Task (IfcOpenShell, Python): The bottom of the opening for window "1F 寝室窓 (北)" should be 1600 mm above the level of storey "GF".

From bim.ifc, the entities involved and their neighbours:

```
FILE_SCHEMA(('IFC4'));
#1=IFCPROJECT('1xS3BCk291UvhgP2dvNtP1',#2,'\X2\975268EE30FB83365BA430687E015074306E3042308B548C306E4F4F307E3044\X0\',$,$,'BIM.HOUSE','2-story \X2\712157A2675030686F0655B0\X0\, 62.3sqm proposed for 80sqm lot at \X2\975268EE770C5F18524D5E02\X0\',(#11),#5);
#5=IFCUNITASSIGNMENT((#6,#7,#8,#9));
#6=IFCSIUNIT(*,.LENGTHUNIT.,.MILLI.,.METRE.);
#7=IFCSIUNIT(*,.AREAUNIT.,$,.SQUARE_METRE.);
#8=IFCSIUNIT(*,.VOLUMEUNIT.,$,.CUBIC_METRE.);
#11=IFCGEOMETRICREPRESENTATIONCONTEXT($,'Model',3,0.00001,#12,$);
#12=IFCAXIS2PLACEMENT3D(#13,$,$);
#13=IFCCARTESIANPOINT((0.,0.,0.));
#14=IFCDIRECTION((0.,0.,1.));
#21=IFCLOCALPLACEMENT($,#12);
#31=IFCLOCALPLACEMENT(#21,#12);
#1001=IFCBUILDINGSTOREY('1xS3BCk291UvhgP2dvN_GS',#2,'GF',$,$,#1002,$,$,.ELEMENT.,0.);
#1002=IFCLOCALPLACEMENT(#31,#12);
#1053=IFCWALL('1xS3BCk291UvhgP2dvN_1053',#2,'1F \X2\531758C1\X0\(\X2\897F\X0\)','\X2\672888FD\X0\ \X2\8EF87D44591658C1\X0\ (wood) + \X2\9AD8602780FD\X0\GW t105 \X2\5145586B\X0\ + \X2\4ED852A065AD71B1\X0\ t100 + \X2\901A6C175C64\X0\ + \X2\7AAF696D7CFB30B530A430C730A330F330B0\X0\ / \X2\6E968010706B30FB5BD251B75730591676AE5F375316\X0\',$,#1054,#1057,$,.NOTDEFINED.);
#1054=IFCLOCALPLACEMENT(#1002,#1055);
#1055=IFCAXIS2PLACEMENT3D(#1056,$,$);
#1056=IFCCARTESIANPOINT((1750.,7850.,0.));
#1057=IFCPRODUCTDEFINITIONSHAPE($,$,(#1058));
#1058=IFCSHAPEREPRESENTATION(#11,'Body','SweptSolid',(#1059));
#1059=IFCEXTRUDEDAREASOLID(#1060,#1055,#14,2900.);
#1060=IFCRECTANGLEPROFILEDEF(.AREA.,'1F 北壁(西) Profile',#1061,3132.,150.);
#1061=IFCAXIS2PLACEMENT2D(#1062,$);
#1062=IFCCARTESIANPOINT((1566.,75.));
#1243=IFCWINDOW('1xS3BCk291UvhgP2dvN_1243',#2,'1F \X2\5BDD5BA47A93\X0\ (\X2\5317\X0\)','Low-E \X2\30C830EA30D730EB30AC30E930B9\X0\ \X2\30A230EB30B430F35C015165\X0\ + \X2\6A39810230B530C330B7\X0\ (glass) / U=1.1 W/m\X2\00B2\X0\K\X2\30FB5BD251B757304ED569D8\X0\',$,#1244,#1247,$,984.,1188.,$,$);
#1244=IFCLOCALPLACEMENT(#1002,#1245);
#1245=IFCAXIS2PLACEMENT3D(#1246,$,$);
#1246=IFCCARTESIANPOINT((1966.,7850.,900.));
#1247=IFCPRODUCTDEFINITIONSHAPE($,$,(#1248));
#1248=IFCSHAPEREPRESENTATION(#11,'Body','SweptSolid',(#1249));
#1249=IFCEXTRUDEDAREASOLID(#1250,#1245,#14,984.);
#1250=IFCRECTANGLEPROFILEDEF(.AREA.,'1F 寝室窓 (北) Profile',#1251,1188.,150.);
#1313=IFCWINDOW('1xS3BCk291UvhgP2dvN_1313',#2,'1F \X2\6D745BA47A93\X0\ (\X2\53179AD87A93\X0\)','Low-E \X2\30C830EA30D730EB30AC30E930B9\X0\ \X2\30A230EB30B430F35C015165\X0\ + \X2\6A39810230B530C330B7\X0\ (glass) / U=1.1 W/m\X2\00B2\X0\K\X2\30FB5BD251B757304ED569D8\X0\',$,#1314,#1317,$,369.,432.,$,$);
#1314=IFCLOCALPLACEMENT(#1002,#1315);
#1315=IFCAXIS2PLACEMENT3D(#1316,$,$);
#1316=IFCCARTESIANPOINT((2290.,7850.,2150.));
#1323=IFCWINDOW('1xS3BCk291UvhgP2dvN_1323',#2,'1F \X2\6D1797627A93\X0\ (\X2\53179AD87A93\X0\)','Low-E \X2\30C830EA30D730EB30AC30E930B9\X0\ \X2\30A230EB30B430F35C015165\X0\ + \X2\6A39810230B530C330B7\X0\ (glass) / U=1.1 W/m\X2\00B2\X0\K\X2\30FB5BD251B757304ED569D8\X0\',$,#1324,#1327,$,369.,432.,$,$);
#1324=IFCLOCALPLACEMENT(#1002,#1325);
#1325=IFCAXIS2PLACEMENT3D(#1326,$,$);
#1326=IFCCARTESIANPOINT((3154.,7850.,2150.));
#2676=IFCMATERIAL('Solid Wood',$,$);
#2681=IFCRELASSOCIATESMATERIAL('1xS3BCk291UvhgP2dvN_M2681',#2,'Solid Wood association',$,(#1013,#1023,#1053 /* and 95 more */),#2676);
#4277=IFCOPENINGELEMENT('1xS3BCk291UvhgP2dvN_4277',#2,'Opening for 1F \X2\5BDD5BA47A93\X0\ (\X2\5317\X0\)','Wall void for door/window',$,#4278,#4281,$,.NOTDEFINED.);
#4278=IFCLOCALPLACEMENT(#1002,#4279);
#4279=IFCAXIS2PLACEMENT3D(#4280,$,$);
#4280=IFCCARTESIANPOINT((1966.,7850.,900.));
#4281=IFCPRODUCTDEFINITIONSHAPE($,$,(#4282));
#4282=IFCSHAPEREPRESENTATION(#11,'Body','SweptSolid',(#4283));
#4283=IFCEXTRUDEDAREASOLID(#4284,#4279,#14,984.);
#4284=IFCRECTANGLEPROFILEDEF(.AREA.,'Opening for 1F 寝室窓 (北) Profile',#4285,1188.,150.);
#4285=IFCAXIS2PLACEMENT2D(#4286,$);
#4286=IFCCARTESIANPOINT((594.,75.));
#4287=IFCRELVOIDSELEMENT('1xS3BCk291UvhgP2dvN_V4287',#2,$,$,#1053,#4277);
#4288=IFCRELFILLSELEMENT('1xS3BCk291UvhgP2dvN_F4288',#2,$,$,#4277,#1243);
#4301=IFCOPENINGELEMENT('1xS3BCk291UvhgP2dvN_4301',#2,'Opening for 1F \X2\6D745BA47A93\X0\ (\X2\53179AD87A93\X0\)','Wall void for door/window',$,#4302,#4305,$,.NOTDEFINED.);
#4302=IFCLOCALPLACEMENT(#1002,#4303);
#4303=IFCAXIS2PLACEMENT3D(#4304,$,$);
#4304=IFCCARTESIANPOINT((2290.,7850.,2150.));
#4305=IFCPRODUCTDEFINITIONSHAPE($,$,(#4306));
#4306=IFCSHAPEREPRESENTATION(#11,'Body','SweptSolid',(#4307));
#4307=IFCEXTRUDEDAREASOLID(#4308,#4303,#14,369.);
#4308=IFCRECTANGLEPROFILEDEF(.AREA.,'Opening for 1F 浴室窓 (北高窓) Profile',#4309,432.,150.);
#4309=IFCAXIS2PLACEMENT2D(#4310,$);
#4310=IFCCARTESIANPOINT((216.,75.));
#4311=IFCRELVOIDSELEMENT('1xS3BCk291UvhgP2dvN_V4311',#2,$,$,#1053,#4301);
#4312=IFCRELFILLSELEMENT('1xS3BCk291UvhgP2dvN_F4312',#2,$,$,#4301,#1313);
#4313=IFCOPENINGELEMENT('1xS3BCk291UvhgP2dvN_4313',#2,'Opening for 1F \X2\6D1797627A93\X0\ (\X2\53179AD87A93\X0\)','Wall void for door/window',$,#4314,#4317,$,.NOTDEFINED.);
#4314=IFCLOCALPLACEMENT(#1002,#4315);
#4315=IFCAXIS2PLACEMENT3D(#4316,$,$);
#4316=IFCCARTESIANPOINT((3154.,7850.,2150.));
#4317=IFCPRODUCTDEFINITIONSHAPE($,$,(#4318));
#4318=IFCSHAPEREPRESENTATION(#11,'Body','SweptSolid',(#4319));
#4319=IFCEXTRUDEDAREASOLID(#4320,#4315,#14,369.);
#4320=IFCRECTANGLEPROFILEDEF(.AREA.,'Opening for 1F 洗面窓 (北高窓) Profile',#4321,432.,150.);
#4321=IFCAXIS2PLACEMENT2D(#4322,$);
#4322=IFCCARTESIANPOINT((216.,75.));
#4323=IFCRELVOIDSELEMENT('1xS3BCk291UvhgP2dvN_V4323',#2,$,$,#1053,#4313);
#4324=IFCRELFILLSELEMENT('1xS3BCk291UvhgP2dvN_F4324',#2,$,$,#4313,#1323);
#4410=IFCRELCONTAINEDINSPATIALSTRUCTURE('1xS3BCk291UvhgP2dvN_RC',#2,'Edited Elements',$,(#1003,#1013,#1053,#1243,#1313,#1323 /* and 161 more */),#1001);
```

```python
import numpy as np
import ifcopenshell
import ifcopenshell.api.geometry
import ifcopenshell.geom
import ifcopenshell.util.element
import ifcopenshell.util.placement
import ifcopenshell.util.shape
import ifcopenshell.util.unit

model = ifcopenshell.open("bim.ifc")
unit_scale = ifcopenshell.util.unit.calculate_unit_scale(model)

window = model.by_guid("1xS3BCk291UvhgP2dvN_1243")
opening = window.FillsVoids[0].RelatingOpeningElement
storey = ifcopenshell.util.element.get_container(window, ifc_class="IfcBuildingStorey")
level = ifcopenshell.util.placement.get_local_placement(storey.ObjectPlacement)[2, 3]

# The opening's origin need not be at the sill, so measure its lowest point.
shape = ifcopenshell.geom.create_shape(ifcopenshell.geom.settings(), opening)
bottom = ifcopenshell.util.shape.get_shape_bottom_elevation(shape, shape.geometry) / unit_scale
dz = level + 1600.0 - bottom

shift = np.array([0.0, 0.0, dz])
# The window is not placed relative to its opening, so move both.
for product in (opening, window):
    matrix = ifcopenshell.util.placement.get_local_placement(product.ObjectPlacement)
    matrix[:3, 3] += shift
    ifcopenshell.api.geometry.edit_object_placement(model, product=product, matrix=matrix, is_si=False)

print(f"moved by {dz * unit_scale:+.3f} m")

model.write("bim_rev.ifc")
```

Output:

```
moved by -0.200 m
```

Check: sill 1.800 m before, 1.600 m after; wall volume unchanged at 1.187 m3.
